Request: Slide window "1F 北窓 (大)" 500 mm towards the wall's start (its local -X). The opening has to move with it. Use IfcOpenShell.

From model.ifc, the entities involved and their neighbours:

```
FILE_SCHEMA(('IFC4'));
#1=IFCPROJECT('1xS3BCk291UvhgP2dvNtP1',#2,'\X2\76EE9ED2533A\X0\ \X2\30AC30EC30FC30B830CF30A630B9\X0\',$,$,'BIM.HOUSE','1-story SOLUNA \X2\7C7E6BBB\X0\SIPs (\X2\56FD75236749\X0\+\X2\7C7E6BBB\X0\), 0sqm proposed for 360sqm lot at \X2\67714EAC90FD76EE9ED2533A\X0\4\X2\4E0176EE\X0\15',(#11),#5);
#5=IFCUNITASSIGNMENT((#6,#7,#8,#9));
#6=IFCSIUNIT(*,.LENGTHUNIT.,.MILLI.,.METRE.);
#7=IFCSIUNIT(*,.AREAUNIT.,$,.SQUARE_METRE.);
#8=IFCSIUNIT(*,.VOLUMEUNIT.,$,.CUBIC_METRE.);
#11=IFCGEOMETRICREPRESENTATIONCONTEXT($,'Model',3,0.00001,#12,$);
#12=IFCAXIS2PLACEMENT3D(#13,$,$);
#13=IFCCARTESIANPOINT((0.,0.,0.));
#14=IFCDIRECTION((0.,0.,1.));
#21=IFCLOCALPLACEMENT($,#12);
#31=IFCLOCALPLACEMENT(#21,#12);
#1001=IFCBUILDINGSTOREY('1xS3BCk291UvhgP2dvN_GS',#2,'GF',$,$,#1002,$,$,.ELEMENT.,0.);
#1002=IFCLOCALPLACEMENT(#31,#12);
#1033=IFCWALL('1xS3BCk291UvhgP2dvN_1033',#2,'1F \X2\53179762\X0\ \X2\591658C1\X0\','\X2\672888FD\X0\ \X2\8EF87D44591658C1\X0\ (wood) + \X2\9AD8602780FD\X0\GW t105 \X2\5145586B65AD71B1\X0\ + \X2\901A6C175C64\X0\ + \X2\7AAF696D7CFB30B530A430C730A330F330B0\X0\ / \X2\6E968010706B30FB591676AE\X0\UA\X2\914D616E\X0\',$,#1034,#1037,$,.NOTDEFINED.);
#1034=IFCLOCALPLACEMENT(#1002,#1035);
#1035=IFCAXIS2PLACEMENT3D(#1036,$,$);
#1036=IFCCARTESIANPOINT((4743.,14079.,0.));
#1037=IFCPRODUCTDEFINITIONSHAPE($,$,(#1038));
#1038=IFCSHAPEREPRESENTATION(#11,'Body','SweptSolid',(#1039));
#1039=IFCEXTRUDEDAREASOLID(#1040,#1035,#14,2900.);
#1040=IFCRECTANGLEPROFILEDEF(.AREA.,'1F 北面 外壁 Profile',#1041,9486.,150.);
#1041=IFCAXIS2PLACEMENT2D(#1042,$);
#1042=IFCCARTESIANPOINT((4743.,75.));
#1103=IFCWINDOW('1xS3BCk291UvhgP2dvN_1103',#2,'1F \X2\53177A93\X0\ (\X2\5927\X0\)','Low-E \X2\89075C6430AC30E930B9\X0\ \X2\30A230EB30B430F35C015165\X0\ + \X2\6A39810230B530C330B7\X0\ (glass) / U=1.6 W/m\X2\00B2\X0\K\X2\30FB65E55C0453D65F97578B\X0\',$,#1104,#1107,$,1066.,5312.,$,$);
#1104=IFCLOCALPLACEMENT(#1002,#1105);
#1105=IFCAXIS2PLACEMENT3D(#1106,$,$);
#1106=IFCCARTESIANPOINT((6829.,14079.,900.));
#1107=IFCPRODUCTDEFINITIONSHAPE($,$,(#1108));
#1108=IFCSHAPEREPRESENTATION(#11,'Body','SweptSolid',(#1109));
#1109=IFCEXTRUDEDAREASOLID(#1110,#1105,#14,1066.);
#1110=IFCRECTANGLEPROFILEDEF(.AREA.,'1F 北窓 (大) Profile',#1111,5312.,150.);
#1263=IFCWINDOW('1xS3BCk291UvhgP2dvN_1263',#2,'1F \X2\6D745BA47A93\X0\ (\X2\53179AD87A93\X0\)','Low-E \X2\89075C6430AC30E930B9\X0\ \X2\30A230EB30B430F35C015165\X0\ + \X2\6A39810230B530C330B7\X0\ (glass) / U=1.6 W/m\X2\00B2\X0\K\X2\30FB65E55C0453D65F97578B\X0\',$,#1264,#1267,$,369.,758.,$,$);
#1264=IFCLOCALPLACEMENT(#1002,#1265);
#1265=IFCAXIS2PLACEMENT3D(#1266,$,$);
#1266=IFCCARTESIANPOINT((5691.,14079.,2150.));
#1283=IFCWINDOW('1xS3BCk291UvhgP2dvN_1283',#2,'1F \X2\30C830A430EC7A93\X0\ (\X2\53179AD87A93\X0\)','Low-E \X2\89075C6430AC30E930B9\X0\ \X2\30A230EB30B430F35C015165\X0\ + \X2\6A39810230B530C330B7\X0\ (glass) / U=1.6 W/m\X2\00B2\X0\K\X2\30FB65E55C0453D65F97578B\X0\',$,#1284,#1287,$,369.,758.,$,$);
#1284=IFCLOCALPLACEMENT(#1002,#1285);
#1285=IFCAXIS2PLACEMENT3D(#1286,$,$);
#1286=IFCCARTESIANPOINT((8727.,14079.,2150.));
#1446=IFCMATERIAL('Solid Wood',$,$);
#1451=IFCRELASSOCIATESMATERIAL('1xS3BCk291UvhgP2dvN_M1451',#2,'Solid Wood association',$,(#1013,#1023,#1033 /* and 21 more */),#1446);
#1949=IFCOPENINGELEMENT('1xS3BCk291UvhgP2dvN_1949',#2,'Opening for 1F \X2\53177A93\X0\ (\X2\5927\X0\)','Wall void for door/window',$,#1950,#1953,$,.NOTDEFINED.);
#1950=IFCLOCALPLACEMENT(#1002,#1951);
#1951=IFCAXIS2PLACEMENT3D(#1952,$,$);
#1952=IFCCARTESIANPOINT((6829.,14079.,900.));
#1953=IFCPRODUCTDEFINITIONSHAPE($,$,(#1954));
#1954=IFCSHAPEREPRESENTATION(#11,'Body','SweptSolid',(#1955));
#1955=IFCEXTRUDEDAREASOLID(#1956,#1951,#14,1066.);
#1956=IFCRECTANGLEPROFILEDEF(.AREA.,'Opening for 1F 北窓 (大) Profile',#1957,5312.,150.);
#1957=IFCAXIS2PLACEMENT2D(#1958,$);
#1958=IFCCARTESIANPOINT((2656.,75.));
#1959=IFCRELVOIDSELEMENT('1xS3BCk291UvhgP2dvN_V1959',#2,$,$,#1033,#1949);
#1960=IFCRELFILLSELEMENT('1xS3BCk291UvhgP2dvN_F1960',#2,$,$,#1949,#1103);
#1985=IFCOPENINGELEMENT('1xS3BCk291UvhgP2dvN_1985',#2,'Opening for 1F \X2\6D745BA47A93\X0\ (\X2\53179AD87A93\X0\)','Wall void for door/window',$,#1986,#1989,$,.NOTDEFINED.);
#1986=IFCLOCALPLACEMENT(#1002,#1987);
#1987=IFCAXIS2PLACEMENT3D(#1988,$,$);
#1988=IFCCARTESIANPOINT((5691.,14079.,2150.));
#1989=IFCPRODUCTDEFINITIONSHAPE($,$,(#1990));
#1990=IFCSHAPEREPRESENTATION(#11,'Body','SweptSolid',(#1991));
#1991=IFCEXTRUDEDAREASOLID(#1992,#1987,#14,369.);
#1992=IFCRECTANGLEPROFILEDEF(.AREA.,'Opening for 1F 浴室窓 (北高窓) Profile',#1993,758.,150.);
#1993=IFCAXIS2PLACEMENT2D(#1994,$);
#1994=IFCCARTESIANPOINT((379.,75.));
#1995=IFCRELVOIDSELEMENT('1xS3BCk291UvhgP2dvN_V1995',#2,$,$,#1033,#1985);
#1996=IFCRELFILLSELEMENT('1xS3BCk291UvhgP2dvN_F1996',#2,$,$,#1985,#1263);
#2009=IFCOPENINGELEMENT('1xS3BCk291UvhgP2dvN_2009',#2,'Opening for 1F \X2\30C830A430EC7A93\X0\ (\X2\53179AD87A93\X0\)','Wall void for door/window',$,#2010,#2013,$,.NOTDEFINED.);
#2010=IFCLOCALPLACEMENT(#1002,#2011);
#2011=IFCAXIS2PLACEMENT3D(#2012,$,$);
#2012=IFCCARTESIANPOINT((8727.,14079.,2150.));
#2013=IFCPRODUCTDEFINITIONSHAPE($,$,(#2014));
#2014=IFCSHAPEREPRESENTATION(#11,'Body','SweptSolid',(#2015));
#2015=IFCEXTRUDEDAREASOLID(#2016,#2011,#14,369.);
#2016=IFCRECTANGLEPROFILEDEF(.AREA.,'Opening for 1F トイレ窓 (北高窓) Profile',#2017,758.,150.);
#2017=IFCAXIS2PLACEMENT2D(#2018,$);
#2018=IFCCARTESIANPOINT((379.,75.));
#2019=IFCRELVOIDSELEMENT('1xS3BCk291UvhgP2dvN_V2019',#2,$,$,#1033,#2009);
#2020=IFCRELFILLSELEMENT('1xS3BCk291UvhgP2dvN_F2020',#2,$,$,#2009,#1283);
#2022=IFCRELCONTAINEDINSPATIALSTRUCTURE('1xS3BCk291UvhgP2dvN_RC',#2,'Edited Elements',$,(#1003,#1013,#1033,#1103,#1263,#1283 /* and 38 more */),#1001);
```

```python
import ifcopenshell
import ifcopenshell.api.geometry
import ifcopenshell.util.placement
import ifcopenshell.util.unit

model = ifcopenshell.open("model.ifc")
unit_scale = ifcopenshell.util.unit.calculate_unit_scale(model)

window = model.by_guid("1xS3BCk291UvhgP2dvN_1103")
opening = window.FillsVoids[0].RelatingOpeningElement
wall = opening.VoidsElements[0].RelatingBuildingElement

wall_matrix = ifcopenshell.util.placement.get_local_placement(wall.ObjectPlacement)
shift = wall_matrix[:3, 0] * -0.5 / unit_scale
before = ifcopenshell.util.placement.get_local_placement(window.ObjectPlacement)[:3, 3].copy()

# The window is not placed relative to its opening, so move both.
for product in (opening, window):
    matrix = ifcopenshell.util.placement.get_local_placement(product.ObjectPlacement)
    matrix[:3, 3] += shift
    ifcopenshell.api.geometry.edit_object_placement(model, product=product, matrix=matrix, is_si=False)

after = ifcopenshell.util.placement.get_local_placement(window.ObjectPlacement)[:3, 3]
print("window moved by", (after - before).round(3) + 0.0)

model.write("model-out.ifc")
```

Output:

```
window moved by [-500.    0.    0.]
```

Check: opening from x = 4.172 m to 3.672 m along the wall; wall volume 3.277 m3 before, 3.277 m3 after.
